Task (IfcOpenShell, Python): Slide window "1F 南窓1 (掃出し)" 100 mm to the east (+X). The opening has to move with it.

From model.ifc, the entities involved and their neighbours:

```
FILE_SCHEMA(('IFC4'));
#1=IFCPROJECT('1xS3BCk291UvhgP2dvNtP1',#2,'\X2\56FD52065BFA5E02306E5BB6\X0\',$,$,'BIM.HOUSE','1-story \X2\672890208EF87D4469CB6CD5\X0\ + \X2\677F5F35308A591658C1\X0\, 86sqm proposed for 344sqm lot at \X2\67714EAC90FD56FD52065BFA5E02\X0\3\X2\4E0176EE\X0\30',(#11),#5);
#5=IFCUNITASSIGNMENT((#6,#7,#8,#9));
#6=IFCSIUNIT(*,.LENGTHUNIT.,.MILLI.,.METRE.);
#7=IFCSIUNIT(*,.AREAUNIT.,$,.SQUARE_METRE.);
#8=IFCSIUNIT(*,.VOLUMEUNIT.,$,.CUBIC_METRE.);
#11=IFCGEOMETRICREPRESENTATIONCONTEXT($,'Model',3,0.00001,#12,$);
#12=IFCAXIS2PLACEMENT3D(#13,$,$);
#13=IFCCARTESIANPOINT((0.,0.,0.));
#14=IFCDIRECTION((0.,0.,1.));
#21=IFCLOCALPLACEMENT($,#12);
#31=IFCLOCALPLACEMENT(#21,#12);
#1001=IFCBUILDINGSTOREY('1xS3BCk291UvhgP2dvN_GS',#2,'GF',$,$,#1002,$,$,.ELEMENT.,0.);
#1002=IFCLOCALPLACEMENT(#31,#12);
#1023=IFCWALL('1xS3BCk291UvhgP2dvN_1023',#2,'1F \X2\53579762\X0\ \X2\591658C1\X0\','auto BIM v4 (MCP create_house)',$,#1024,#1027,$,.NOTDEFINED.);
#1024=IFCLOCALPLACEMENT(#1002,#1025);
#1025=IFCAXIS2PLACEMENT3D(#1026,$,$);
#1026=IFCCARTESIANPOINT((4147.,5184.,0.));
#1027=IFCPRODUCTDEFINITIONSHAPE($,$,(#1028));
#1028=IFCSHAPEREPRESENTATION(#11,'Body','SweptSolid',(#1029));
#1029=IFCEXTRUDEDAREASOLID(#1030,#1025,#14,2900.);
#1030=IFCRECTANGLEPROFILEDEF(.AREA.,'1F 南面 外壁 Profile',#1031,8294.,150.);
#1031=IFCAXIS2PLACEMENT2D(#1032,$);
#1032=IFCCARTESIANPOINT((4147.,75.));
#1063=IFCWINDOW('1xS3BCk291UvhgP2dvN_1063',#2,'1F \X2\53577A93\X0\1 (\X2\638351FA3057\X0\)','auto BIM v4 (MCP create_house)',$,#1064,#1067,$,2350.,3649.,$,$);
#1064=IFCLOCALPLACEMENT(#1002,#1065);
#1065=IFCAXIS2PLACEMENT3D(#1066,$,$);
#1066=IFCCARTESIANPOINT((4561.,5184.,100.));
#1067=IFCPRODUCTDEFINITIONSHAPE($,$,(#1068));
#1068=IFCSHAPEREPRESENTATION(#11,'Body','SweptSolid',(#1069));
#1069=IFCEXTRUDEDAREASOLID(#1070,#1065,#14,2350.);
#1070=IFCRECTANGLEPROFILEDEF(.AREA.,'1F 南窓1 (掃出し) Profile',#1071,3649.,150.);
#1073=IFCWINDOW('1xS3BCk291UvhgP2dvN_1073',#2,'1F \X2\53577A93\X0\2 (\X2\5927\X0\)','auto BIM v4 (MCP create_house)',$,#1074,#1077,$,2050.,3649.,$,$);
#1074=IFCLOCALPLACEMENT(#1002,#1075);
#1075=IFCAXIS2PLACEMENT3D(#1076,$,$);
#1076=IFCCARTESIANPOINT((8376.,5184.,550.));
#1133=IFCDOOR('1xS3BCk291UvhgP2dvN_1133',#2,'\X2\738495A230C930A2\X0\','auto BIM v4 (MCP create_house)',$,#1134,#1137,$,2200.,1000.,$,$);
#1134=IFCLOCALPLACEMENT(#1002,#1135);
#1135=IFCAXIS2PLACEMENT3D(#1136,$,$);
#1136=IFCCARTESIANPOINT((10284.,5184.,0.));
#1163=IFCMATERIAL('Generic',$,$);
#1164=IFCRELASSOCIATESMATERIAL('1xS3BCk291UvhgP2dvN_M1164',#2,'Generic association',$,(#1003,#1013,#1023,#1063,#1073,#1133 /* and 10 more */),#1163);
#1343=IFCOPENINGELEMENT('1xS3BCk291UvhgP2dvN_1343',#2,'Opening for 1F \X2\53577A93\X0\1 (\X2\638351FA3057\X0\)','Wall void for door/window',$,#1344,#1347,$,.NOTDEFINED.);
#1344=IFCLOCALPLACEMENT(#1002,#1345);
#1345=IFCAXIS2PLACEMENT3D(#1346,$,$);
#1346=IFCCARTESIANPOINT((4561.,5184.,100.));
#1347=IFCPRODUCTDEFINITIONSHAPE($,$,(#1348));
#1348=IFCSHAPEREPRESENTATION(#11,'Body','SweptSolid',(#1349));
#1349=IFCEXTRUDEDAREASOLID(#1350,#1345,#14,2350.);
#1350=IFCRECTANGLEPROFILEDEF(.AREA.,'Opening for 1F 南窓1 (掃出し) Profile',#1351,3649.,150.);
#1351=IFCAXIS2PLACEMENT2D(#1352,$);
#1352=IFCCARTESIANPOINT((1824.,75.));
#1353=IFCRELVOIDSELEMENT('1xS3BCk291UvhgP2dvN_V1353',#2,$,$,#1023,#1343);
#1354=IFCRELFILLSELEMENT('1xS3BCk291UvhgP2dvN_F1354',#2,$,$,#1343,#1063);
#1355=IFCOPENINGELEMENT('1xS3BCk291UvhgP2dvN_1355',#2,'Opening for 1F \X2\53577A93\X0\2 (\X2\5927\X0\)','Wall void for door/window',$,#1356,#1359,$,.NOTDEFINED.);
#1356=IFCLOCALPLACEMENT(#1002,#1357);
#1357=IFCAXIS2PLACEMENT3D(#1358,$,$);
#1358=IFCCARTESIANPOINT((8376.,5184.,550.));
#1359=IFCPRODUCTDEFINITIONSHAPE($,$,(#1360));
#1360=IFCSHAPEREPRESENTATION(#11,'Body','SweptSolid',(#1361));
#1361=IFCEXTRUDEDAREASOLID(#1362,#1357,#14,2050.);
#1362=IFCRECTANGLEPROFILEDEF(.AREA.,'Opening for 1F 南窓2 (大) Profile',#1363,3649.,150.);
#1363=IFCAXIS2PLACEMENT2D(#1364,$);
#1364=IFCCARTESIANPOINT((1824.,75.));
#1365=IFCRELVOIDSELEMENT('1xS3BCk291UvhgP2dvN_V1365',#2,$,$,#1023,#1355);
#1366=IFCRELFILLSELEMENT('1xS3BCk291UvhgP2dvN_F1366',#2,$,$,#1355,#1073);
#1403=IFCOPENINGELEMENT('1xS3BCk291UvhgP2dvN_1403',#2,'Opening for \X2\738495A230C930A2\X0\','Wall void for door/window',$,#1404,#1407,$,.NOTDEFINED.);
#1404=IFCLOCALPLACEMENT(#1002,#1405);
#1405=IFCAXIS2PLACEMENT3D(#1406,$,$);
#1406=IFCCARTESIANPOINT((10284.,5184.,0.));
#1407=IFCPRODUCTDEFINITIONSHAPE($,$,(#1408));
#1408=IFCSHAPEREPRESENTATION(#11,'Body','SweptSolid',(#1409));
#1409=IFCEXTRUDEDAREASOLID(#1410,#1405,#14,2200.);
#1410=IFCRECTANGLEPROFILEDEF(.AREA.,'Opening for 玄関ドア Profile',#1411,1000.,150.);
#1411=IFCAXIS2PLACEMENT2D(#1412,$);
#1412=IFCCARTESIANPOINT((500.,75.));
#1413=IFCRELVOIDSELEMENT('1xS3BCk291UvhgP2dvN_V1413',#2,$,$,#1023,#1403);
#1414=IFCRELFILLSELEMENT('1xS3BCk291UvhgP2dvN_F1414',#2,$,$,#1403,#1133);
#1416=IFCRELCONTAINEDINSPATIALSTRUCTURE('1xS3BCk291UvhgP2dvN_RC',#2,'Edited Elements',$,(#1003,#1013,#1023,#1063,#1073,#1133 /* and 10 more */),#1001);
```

```python
import ifcopenshell
import ifcopenshell.api.geometry
import ifcopenshell.util.placement
import ifcopenshell.util.unit

model = ifcopenshell.open("model.ifc")
unit_scale = ifcopenshell.util.unit.calculate_unit_scale(model)

window = model.by_id(1063)
opening = window.FillsVoids[0].RelatingOpeningElement
wall = opening.VoidsElements[0].RelatingBuildingElement

wall_matrix = ifcopenshell.util.placement.get_local_placement(wall.ObjectPlacement)
shift = wall_matrix[:3, 0] * 0.1 / unit_scale
before = ifcopenshell.util.placement.get_local_placement(window.ObjectPlacement)[:3, 3].copy()

# The window is not placed relative to its opening, so move both.
for product in (opening, window):
    matrix = ifcopenshell.util.placement.get_local_placement(product.ObjectPlacement)
    matrix[:3, 3] += shift
    ifcopenshell.api.geometry.edit_object_placement(model, product=product, matrix=matrix, is_si=False)

after = ifcopenshell.util.placement.get_local_placement(window.ObjectPlacement)[:3, 3]
print("window moved by", (after - before).round(3) + 0.0)

model.write("model_updated.ifc")
```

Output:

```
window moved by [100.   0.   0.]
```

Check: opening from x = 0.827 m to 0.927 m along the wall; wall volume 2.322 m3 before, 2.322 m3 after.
